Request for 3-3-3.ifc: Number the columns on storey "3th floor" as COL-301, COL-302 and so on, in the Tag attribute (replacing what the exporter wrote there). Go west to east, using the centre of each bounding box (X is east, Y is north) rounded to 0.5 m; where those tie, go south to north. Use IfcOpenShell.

First a look at what the model holds.

```python
import ifcopenshell
import ifcopenshell.util.element
import ifcopenshell.util.placement

model = ifcopenshell.open("3-3-3.ifc")
print(model.schema)
storey = next(s for s in model.by_type("IfcBuildingStorey") if s.Name == "3th floor")
columns = [e for e in ifcopenshell.util.element.get_decomposition(storey) if e.is_a("IfcColumn")]
for e in sorted(columns, key=lambda e: e.id()):
    origin = ifcopenshell.util.placement.get_local_placement(e.ObjectPlacement)[:3, 3]
    print(e.id(), e.Tag, e.Name, origin.round(2) + 0.0, sep=" | ")
```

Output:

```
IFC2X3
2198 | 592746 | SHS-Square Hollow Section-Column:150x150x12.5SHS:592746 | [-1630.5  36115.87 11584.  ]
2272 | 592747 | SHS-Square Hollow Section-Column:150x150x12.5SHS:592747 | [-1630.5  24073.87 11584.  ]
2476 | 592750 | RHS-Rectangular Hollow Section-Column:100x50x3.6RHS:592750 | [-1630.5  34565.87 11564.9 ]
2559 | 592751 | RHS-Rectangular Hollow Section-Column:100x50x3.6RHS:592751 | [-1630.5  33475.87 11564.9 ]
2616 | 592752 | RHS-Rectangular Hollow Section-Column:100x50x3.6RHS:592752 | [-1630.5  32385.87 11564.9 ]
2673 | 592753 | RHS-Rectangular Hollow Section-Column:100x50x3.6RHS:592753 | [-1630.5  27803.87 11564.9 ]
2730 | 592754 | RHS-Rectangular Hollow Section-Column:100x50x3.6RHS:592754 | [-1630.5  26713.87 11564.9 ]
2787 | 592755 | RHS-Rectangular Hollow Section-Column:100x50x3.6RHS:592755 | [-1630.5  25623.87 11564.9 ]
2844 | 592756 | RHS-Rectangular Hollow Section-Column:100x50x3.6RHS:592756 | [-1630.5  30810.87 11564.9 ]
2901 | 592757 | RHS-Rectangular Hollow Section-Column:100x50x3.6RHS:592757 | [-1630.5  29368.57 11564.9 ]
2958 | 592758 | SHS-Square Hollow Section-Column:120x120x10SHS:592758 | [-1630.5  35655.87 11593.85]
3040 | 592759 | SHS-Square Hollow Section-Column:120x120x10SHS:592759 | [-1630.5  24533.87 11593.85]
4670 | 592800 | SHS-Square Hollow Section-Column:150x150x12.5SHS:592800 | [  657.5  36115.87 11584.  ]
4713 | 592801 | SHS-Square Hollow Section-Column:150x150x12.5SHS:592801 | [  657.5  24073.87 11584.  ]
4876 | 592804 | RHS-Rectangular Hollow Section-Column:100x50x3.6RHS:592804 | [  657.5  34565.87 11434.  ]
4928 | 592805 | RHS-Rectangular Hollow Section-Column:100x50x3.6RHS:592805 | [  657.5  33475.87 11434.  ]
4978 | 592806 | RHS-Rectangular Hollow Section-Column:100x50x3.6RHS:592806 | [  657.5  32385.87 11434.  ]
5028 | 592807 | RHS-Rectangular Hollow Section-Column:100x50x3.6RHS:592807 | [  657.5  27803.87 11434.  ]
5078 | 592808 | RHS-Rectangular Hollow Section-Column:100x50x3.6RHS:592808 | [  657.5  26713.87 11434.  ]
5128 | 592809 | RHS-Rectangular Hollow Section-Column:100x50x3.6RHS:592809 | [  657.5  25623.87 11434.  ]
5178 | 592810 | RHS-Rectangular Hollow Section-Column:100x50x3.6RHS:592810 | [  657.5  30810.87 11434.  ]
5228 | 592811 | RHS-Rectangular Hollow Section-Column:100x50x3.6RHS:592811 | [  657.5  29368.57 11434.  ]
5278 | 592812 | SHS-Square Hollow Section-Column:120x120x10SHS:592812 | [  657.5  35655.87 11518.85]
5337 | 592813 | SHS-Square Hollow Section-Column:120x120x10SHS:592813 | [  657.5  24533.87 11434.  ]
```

```python
import ifcopenshell
import ifcopenshell.geom
import ifcopenshell.util.element
import ifcopenshell.util.shape

model = ifcopenshell.open("3-3-3.ifc")
settings = ifcopenshell.geom.settings()
settings.set("use-world-coords", True)


def centre(element):
    shape = ifcopenshell.geom.create_shape(settings, element)
    return ifcopenshell.util.shape.get_bbox_centroid(shape.geometry)


storey = next(s for s in model.by_type("IfcBuildingStorey") if s.Name == "3th floor")
columns = [e for e in ifcopenshell.util.element.get_decomposition(storey) if e.is_a("IfcColumn")]

# Insertion points can sit at a corner or the storey origin, so sort by the geometry (in metres).
centres = {e: centre(e) for e in columns}
columns.sort(key=lambda e: (round(centres[e][0] / 0.5), centres[e][1]))

for i, e in enumerate(columns, start=1):
    number = f"COL-3{i:02d}"
    e.Tag = number
    print(e.id(), number)

model.write("3-3-3_v2.ifc")
```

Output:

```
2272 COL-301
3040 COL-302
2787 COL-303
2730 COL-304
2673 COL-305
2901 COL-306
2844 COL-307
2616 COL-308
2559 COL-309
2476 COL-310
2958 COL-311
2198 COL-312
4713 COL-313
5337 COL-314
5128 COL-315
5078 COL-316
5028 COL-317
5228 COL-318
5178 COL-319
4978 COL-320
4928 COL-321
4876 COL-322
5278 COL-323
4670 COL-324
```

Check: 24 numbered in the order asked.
